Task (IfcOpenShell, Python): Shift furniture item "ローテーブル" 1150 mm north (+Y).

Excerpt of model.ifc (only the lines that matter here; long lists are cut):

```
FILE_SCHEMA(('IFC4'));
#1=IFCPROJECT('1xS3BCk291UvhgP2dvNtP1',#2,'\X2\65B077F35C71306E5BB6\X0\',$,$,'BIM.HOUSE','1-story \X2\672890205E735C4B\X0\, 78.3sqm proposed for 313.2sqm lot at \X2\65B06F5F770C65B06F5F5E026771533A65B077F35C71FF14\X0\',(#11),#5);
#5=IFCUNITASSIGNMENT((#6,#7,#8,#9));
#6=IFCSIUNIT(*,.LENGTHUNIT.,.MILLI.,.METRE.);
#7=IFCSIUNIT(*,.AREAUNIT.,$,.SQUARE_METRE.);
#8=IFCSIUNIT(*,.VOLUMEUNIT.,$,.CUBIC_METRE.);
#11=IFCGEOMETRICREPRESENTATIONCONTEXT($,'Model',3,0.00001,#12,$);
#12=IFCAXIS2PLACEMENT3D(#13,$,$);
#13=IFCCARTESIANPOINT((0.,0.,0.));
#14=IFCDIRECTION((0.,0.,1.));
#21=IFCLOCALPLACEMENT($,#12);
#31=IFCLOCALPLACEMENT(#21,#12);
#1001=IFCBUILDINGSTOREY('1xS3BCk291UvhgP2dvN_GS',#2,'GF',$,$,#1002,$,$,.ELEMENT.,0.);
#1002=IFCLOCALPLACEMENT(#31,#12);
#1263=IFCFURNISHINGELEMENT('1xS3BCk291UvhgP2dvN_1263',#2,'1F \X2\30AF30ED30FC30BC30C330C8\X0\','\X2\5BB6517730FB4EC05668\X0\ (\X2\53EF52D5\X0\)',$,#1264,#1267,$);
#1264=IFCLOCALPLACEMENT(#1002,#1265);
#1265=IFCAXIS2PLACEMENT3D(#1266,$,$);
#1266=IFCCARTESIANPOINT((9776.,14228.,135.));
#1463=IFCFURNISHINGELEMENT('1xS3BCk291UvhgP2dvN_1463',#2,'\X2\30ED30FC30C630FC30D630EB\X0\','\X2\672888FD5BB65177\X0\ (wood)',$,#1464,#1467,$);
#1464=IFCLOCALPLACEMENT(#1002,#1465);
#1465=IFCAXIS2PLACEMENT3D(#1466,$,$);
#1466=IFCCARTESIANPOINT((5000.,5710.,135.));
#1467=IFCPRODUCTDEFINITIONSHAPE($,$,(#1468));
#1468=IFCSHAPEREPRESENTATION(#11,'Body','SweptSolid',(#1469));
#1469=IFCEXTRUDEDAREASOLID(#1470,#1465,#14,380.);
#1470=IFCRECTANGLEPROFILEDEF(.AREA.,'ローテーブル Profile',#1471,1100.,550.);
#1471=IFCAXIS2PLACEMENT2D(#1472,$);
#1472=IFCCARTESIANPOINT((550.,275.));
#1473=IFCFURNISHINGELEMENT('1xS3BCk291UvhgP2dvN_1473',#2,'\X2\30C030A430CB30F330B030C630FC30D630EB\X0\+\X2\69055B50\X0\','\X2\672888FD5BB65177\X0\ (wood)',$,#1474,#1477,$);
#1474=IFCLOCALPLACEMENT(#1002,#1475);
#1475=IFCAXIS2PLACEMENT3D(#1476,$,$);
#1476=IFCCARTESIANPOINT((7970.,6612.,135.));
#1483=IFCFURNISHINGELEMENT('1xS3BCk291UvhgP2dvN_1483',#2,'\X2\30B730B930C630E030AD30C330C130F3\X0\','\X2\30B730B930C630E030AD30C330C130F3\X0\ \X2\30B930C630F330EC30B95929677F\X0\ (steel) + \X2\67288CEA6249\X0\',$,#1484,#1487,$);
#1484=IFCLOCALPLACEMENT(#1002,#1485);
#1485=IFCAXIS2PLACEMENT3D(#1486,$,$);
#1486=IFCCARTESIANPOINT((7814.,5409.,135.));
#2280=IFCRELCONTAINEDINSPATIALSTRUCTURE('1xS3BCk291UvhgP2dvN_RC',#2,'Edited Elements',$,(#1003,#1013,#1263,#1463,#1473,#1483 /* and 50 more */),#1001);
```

```python
import ifcopenshell
import ifcopenshell.api.geometry
import ifcopenshell.util.placement
import ifcopenshell.util.unit

model = ifcopenshell.open("model.ifc")
unit_scale = ifcopenshell.util.unit.calculate_unit_scale(model)

item = model.by_id(1463)
matrix = ifcopenshell.util.placement.get_local_placement(item.ObjectPlacement)
matrix[1, 3] += 1.15 / unit_scale
ifcopenshell.api.geometry.edit_object_placement(model, product=item, matrix=matrix, is_si=False)

print(ifcopenshell.util.placement.get_local_placement(item.ObjectPlacement).round(3) + 0.0)

model.write("model_rev.ifc")
```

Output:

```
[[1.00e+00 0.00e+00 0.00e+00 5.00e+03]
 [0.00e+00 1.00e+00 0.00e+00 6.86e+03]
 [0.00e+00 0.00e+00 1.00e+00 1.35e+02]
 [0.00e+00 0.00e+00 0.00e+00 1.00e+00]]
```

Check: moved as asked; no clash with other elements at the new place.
